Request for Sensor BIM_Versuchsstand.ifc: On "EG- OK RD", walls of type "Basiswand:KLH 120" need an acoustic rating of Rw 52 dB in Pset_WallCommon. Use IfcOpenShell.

First a look at what the model holds.

```python
import ifcopenshell
import ifcopenshell.util.element

model = ifcopenshell.open("Sensor BIM_Versuchsstand.ifc")
print(model.schema)
storey = next(s for s in model.by_type("IfcBuildingStorey") if s.Name == "EG- OK RD")
walls = [e for e in ifcopenshell.util.element.get_decomposition(storey) if e.is_a("IfcWall")]
seen = {}
for e in walls:
    element_type = ifcopenshell.util.element.get_type(e)
    key = (element_type.Name if element_type != e and element_type else None, ifcopenshell.util.element.get_pset(e, "Pset_WallCommon", "AcousticRating"))
    seen[key] = seen.get(key, 0) + 1
for (name, value), count in sorted(seen.items(), key=str):
    print(count, "x", name, "|", value)
```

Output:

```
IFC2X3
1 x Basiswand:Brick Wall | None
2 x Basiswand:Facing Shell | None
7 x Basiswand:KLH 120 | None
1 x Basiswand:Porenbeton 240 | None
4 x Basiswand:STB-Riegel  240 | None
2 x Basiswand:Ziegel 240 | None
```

```python
import ifcopenshell
import ifcopenshell.api.pset
import ifcopenshell.util.element

model = ifcopenshell.open("Sensor BIM_Versuchsstand.ifc")

storey = next(s for s in model.by_type("IfcBuildingStorey") if s.Name == "EG- OK RD")
walls = [e for e in ifcopenshell.util.element.get_decomposition(storey) if e.is_a("IfcWall")]

count = 0
for e in walls:
    element_type = ifcopenshell.util.element.get_type(e)
    if element_type in (None, e) or element_type.Name != "Basiswand:KLH 120":
        continue
    # add_pset returns the element's existing set when there is one.
    pset = ifcopenshell.api.pset.add_pset(model, product=e, name="Pset_WallCommon")
    ifcopenshell.api.pset.edit_pset(model, pset=pset, properties={"AcousticRating": "Rw 52 dB"})
    count += 1

print(count, "walls updated")

model.write("Sensor BIM_Versuchsstand_edited.ifc")
```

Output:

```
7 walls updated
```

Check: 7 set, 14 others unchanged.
